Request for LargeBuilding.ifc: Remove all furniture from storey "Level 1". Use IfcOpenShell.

First a look at what the model holds.

```python
import ifcopenshell
import ifcopenshell.util.element

model = ifcopenshell.open("LargeBuilding.ifc")
print(model.schema)
storey = next(s for s in model.by_type("IfcBuildingStorey") if s.Name == "Level 1")
furniture = [e for e in ifcopenshell.util.element.get_decomposition(storey) if e.is_a("IfcFurnishingElement")]
seen = {}
for e in furniture:
    element_type = ifcopenshell.util.element.get_type(e)
    name = element_type.Name if element_type not in (None, e) else None
    seen[name] = seen.get(name, 0) + 1
for name, count in sorted(seen.items(), key=str):
    print(count, "x", name)
```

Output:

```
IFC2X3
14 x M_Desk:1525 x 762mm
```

```python
import ifcopenshell
import ifcopenshell.api.root
import ifcopenshell.util.element

model = ifcopenshell.open("LargeBuilding.ifc")

storey = next(s for s in model.by_type("IfcBuildingStorey") if s.Name == "Level 1")
furniture = [e for e in ifcopenshell.util.element.get_decomposition(storey) if e.is_a("IfcFurnishingElement")]

for e in furniture:
    ifcopenshell.api.root.remove_product(model, product=e)
print(len(furniture), "removed")

model.write("LargeBuilding_updated.ifc")
```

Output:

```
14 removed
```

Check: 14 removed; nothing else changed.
